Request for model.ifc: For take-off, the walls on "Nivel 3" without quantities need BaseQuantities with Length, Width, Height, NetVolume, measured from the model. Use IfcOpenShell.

First a look at what the model holds.

```python
import ifcopenshell
import ifcopenshell.util.element
import ifcopenshell.util.unit

model = ifcopenshell.open("model.ifc")
print(model.schema)
for unit_type in ("LENGTHUNIT", "AREAUNIT", "VOLUMEUNIT"):
    print(unit_type, ifcopenshell.util.unit.calculate_unit_scale(model, unit_type))
storey = next(s for s in model.by_type("IfcBuildingStorey") if s.Name == "Nivel 3")
walls = [e for e in ifcopenshell.util.element.get_decomposition(storey) if e.is_a("IfcWall")]
for e in sorted(walls, key=lambda e: e.id()):
    print(e.id(), e.is_a(), e.Name, list(ifcopenshell.util.element.get_psets(e, qtos_only=True)), sep=" | ")
```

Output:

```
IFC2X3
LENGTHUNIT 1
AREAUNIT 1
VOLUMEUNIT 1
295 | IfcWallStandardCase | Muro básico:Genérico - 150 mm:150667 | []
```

```python
import ifcopenshell
import ifcopenshell.api.pset
import ifcopenshell.geom
import ifcopenshell.util.element
import ifcopenshell.util.shape
import ifcopenshell.util.unit

model = ifcopenshell.open("model.ifc")
unit_scale = ifcopenshell.util.unit.calculate_unit_scale(model)
volume_scale = ifcopenshell.util.unit.calculate_unit_scale(model, "VOLUMEUNIT")
settings = ifcopenshell.geom.settings()

storey = next(s for s in model.by_type("IfcBuildingStorey") if s.Name == "Nivel 3")
walls = [e for e in ifcopenshell.util.element.get_decomposition(storey) if e.is_a("IfcWall")]

for e in sorted(walls, key=lambda e: e.id()):
    if ifcopenshell.util.element.get_psets(e, qtos_only=True, should_inherit=False):
        continue
    # Geometry comes back in metres, in the element's own axes.
    shape = ifcopenshell.geom.create_shape(settings, e)
    values = {
        "Length": ifcopenshell.util.shape.get_x(shape.geometry) / unit_scale,
        "Width": ifcopenshell.util.shape.get_y(shape.geometry) / unit_scale,
        "Height": ifcopenshell.util.shape.get_z(shape.geometry) / unit_scale,
        "NetVolume": ifcopenshell.util.shape.get_volume(shape.geometry) / volume_scale,
    }
    qto = ifcopenshell.api.pset.add_qto(model, product=e, name="BaseQuantities")
    ifcopenshell.api.pset.edit_qto(model, qto=qto, properties=values)
    print(e.id(), {k: round(v, 3) for k, v in values.items()})

model.write("model_v2.ifc")
```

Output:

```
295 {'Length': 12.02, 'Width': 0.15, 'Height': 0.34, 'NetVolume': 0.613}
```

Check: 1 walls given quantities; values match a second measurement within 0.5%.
